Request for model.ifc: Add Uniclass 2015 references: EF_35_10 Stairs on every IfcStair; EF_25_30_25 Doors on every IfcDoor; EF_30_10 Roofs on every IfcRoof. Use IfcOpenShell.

First a look at what the model holds.

```python
import ifcopenshell

model = ifcopenshell.open("model.ifc")
print(model.schema)
print("classifications:", [c.Name for c in model.by_type("IfcClassification")])
for ifc_class in ("IfcDoor", "IfcRoof", "IfcStair", "IfcWall", "IfcWindow"):
    print(ifc_class, len(model.by_type(ifc_class)))
```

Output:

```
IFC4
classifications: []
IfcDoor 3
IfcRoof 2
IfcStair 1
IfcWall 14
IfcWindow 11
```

```python
import ifcopenshell
import ifcopenshell.api.classification

model = ifcopenshell.open("model.ifc")

system = ifcopenshell.api.classification.add_classification(model, classification="Uniclass 2015")

codes = {
    "IfcStair": ("EF_35_10", "Stairs"),
    "IfcDoor": ("EF_25_30_25", "Doors"),
    "IfcRoof": ("EF_30_10", "Roofs"),
}
for ifc_class, (code, name) in codes.items():
    products = model.by_type(ifc_class)
    ifcopenshell.api.classification.add_reference(
        model, products=products, classification=system, identification=code, name=name
    )
    print(code, len(products))

model.write("model-out.ifc")
```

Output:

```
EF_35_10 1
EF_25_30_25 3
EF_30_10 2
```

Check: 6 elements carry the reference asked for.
